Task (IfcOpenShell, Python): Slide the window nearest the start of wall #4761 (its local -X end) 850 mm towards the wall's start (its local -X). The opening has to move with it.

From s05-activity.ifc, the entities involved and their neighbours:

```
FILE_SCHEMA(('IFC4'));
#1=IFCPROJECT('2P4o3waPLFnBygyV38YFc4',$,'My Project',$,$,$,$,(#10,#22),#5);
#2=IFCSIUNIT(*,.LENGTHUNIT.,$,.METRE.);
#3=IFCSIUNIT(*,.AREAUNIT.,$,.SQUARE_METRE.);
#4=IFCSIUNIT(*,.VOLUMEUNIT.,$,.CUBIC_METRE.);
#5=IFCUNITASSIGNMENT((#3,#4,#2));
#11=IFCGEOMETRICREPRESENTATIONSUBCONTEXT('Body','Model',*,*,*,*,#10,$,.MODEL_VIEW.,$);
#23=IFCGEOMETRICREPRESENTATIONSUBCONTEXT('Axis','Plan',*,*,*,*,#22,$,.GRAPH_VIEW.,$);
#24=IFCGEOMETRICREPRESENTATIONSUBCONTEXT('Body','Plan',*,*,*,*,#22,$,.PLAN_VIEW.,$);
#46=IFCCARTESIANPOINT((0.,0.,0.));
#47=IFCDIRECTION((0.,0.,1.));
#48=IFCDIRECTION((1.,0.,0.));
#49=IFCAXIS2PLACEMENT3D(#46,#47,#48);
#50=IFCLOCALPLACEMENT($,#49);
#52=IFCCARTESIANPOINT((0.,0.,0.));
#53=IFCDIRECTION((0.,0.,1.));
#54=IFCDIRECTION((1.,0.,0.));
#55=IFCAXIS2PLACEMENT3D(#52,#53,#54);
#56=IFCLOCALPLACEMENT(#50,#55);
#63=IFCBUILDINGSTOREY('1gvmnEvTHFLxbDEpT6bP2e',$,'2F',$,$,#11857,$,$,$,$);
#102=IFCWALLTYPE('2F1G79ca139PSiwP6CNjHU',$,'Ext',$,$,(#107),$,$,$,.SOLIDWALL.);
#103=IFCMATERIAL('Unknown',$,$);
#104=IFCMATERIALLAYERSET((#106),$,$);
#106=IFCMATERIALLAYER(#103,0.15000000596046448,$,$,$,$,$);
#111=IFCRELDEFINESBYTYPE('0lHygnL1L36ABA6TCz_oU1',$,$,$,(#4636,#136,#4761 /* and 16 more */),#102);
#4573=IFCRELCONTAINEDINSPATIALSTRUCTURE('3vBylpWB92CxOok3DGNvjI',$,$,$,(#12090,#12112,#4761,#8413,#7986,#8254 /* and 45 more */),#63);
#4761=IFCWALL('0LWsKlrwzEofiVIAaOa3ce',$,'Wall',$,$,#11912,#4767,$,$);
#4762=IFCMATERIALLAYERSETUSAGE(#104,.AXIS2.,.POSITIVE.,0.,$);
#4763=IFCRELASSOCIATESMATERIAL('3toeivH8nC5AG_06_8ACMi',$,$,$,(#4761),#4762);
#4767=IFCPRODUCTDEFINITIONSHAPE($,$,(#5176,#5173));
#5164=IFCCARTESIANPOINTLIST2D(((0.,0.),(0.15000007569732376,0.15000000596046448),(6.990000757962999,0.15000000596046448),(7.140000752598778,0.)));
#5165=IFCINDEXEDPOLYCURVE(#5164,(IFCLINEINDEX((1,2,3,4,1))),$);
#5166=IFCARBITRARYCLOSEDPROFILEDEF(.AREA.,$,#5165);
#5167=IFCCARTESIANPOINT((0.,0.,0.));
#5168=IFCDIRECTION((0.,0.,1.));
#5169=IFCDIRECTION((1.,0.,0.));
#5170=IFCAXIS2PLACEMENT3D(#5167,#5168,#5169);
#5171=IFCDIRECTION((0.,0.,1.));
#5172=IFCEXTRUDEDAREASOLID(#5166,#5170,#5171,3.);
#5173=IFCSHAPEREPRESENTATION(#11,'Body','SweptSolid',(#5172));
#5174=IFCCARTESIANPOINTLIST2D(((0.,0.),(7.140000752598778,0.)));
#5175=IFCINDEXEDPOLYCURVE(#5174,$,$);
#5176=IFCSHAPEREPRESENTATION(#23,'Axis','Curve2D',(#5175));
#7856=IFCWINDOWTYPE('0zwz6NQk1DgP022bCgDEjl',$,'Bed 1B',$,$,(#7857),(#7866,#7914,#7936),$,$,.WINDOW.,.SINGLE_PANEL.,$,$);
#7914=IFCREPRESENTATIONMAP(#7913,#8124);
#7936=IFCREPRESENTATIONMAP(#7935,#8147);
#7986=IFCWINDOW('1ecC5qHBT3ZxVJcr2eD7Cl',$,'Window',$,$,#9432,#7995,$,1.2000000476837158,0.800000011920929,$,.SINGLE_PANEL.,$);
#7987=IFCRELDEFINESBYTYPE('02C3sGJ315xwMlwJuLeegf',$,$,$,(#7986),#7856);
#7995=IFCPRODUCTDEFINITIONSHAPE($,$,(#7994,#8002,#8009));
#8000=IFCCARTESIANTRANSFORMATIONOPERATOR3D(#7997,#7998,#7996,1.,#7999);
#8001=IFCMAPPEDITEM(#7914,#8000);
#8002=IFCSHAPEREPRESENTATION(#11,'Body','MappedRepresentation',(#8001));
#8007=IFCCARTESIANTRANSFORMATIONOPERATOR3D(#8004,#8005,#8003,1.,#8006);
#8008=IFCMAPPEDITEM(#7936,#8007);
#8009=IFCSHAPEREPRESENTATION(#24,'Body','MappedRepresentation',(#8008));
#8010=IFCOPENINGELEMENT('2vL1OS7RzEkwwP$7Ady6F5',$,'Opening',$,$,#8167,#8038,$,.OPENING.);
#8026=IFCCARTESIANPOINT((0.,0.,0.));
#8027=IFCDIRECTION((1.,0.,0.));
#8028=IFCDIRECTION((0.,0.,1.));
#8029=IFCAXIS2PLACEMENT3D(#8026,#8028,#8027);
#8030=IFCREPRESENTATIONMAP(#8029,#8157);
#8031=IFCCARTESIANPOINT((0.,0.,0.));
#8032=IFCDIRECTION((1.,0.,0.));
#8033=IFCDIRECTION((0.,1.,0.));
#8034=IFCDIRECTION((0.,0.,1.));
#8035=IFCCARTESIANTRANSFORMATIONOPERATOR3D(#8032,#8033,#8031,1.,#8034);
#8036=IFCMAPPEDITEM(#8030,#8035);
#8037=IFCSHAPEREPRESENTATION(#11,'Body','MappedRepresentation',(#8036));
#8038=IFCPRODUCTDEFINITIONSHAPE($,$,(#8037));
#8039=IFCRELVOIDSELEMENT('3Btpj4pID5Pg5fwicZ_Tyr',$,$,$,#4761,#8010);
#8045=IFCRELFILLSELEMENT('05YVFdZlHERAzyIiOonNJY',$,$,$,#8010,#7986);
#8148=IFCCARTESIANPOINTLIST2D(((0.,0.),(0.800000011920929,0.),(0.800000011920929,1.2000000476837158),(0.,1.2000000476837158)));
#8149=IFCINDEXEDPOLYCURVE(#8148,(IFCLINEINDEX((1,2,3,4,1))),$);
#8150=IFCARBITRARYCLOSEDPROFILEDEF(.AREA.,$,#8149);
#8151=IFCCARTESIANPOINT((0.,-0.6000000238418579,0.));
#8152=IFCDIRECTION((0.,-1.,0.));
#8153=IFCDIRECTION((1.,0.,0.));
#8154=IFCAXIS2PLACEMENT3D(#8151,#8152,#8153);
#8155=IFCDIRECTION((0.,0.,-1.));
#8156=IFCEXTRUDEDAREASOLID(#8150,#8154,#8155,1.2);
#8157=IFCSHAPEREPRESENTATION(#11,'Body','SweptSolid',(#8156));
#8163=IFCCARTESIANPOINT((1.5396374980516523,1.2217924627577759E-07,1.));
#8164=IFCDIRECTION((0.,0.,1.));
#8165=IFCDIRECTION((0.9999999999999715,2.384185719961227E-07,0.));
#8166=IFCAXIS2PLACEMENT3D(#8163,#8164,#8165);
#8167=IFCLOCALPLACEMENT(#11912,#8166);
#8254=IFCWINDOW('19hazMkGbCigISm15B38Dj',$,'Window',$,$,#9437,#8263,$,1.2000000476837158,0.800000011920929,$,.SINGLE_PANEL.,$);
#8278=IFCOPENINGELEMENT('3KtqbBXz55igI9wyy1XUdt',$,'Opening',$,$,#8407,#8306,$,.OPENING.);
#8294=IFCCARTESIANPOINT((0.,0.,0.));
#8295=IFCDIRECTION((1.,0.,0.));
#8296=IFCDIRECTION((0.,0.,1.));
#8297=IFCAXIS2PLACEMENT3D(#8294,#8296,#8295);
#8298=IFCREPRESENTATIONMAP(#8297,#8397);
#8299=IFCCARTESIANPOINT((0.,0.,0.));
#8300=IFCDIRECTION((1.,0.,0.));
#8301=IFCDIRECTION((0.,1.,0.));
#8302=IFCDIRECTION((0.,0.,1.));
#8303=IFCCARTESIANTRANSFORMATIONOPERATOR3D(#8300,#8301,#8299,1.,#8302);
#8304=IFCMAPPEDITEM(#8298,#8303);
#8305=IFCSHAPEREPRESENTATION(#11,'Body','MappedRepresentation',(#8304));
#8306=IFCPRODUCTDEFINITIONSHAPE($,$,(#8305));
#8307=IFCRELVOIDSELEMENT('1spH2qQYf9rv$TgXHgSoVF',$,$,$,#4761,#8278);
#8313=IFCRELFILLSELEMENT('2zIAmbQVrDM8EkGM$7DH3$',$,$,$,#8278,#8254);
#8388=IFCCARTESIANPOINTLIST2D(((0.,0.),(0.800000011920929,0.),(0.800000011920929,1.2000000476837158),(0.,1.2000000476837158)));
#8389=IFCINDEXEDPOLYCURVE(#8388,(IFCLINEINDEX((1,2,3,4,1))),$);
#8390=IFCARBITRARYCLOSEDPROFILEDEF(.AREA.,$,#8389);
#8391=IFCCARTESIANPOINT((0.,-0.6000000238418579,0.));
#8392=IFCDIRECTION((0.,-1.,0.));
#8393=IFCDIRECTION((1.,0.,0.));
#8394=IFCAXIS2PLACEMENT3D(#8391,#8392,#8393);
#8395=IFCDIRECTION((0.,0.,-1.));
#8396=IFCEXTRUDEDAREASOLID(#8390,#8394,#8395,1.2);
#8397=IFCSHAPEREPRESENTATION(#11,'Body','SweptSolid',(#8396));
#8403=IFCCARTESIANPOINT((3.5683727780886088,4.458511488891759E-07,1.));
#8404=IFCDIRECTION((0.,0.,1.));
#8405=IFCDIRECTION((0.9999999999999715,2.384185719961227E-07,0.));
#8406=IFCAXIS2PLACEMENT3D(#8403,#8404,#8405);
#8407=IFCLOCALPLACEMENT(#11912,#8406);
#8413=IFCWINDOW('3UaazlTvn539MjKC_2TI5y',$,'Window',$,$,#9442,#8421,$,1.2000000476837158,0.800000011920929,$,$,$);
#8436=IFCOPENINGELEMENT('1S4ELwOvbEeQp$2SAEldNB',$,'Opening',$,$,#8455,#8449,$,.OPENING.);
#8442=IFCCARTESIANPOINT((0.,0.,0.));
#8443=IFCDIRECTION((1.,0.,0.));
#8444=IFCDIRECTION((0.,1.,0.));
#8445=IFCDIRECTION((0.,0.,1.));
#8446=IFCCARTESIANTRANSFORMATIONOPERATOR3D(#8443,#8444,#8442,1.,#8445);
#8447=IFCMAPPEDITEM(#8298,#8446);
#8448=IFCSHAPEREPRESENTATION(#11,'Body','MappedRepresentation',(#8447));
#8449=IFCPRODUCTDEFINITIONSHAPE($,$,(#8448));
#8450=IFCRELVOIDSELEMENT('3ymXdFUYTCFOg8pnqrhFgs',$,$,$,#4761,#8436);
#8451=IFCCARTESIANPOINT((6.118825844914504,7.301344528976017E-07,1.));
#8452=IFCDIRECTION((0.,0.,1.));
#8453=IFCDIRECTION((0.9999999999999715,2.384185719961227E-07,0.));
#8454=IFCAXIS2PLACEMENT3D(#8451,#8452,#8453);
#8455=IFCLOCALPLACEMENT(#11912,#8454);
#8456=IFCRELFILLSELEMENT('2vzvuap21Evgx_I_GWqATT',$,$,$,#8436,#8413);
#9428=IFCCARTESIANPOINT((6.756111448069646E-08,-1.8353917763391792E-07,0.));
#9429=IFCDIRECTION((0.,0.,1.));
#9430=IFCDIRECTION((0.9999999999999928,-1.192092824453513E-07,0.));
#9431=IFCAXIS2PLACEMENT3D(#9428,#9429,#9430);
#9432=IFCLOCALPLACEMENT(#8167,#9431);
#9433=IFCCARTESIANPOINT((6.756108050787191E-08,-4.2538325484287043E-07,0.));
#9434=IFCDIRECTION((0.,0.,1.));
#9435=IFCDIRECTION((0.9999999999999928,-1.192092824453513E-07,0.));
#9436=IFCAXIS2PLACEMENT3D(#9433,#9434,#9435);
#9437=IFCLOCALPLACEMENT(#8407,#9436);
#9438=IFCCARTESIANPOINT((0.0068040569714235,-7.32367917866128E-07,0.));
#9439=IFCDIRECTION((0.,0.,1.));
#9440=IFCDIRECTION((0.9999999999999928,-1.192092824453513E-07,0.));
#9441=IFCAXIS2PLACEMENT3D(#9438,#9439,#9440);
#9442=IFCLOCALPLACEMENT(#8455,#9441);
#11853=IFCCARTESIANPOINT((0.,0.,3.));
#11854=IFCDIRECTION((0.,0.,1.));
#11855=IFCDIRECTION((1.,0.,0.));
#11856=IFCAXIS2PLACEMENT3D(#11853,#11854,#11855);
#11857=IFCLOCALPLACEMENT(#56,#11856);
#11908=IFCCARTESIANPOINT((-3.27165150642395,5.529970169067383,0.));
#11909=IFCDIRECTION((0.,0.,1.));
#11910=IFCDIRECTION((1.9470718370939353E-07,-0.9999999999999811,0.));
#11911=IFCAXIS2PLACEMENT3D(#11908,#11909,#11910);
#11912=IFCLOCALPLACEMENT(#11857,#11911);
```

```python
import ifcopenshell
import ifcopenshell.api.geometry
import ifcopenshell.util.placement

model = ifcopenshell.open("s05-activity.ifc")

window = model.by_guid("1ecC5qHBT3ZxVJcr2eD7Cl")
opening = window.FillsVoids[0].RelatingOpeningElement
wall = opening.VoidsElements[0].RelatingBuildingElement

wall_matrix = ifcopenshell.util.placement.get_local_placement(wall.ObjectPlacement)
shift = wall_matrix[:3, 0] * -0.85
before = ifcopenshell.util.placement.get_local_placement(window.ObjectPlacement)[:3, 3].copy()

# The window is placed relative to its opening, so it follows when the opening moves.
matrix = ifcopenshell.util.placement.get_local_placement(opening.ObjectPlacement)
matrix[:3, 3] += shift
ifcopenshell.api.geometry.edit_object_placement(
    model, product=opening, matrix=matrix, is_si=False, should_transform_children=True
)

after = ifcopenshell.util.placement.get_local_placement(window.ObjectPlacement)[:3, 3]
print("window moved by", (after - before).round(3) + 0.0)

model.write("s05-activity_edited.ifc")
```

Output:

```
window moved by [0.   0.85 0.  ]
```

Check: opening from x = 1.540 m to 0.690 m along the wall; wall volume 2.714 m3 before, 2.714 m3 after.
